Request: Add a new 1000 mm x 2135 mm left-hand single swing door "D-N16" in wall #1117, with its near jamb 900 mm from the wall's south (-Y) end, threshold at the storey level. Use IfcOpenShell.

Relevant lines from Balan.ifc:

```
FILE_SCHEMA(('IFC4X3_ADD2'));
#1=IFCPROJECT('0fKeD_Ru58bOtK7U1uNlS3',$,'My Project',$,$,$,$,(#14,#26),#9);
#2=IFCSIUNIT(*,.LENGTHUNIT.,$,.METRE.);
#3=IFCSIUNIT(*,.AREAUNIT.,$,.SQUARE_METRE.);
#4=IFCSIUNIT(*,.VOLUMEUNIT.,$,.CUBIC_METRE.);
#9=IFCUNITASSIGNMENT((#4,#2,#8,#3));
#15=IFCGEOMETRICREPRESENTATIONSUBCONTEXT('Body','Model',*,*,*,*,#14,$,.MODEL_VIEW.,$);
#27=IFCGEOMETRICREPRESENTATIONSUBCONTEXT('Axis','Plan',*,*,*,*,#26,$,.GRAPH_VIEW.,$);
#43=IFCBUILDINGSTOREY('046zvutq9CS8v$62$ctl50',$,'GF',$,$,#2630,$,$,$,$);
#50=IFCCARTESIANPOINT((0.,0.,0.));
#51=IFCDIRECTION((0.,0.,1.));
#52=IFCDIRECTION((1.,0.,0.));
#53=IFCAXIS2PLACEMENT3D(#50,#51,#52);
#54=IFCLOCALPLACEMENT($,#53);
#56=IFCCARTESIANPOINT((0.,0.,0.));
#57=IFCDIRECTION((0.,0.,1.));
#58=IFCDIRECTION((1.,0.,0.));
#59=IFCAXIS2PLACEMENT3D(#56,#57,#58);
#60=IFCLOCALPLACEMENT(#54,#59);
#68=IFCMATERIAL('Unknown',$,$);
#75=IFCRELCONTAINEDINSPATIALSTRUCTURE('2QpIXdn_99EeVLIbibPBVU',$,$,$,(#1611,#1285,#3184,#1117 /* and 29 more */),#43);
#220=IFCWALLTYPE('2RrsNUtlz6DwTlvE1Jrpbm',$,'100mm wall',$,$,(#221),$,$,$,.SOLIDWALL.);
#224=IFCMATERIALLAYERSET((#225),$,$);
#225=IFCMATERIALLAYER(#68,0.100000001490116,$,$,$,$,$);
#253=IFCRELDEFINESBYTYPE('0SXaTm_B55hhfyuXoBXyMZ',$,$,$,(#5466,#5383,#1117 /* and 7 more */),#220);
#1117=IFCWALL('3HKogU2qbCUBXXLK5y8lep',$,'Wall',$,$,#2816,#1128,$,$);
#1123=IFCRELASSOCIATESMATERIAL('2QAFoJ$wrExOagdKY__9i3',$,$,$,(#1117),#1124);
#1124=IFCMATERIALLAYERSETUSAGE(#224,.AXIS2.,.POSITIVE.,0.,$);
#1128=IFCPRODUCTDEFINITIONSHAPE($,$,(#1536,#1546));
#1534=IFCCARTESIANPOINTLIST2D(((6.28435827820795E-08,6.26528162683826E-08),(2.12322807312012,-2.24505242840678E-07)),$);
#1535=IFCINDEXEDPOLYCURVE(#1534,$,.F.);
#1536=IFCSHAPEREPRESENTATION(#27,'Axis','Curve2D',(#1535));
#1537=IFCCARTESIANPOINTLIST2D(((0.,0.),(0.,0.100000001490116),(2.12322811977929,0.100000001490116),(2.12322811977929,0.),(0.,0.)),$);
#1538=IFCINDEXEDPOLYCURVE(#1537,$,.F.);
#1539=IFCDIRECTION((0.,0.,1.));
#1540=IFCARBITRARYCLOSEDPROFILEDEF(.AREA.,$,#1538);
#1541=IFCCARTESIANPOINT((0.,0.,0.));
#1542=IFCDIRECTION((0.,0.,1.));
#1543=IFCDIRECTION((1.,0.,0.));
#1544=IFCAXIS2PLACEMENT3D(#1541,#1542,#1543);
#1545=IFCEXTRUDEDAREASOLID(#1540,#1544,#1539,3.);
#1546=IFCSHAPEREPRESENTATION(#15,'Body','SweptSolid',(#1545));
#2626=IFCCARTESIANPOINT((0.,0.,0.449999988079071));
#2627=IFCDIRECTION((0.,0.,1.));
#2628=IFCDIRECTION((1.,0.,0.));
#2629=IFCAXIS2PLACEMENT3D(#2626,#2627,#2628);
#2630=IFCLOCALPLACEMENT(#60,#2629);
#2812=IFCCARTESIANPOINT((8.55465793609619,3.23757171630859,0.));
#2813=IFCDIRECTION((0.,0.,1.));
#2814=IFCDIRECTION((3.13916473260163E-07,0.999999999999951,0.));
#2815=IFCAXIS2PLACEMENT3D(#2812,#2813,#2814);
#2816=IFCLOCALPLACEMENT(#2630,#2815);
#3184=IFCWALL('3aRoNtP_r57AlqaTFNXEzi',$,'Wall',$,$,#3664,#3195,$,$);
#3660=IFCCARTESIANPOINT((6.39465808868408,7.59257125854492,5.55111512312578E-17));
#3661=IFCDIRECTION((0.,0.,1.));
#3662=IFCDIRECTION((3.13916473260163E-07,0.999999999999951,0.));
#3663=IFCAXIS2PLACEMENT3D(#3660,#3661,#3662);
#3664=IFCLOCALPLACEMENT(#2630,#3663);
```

```python
import numpy as np
import ifcopenshell
import ifcopenshell.api.feature
import ifcopenshell.api.geometry
import ifcopenshell.api.root
import ifcopenshell.api.spatial
import ifcopenshell.geom
import ifcopenshell.util.element
import ifcopenshell.util.placement
import ifcopenshell.util.representation
import ifcopenshell.util.shape
import ifcopenshell.util.unit

model = ifcopenshell.open("Balan.ifc")
unit_scale = ifcopenshell.util.unit.calculate_unit_scale(model)
settings = ifcopenshell.geom.settings()


def volume(element):
    """Net volume in cubic metres, openings subtracted."""
    shape = ifcopenshell.geom.create_shape(settings, element)
    return ifcopenshell.util.shape.get_volume(shape.geometry)


wall = model.by_guid("3HKogU2qbCUBXXLK5y8lep")
storey = ifcopenshell.util.element.get_container(wall, ifc_class="IfcBuildingStorey")
context = ifcopenshell.util.representation.get_context(model, "Model", "Body", "MODEL_VIEW")
before = volume(wall)

width, height, from_end, sill = 1, 2.135, 0.9, 0.0  # metres

# The wall runs along its own X axis, and the end named is its -X end.
wall_shape = ifcopenshell.geom.create_shape(settings, wall)
x, y, z = ifcopenshell.util.shape.get_vertices(wall_shape.geometry).T
start = x.min() + from_end
face, thickness = float(y.min()), float(y.max() - y.min())
wall_matrix = ifcopenshell.util.placement.get_local_placement(wall.ObjectPlacement)
level = ifcopenshell.util.placement.get_local_placement(storey.ObjectPlacement)[2, 3]


def in_wall(x, y):
    """Placement at x, y metres in the wall's axes, at sill height."""
    matrix = wall_matrix.copy()
    matrix[:, 3] = wall_matrix @ np.array([x / unit_scale, y / unit_scale, 0.0, 1.0])
    matrix[2, 3] = level + sill / unit_scale
    return matrix


# Opening: a box that overshoots both wall faces by 50 mm.
opening = ifcopenshell.api.root.create_entity(model, ifc_class="IfcOpeningElement", predefined_type="OPENING")
box = ifcopenshell.api.geometry.add_wall_representation(
    model, context=context, length=width, height=height, thickness=thickness + 0.1
)
ifcopenshell.api.geometry.assign_representation(model, product=opening, representation=box)
ifcopenshell.api.geometry.edit_object_placement(model, product=opening, matrix=in_wall(start, face - 0.05), is_si=False)
ifcopenshell.api.feature.add_feature(model, feature=opening, element=wall)

door = ifcopenshell.api.root.create_entity(model, ifc_class="IfcDoor", name="D-N16", predefined_type="DOOR")
door.OverallWidth, door.OverallHeight = width / unit_scale, height / unit_scale
door.OperationType = "SINGLE_SWING_LEFT"
body = ifcopenshell.api.geometry.add_door_representation(
    model,
    context=context,
    overall_width=door.OverallWidth,
    overall_height=door.OverallHeight,
    operation_type="SINGLE_SWING_LEFT",
    lining_properties={"LiningDepth": thickness / unit_scale, "ThresholdDepth": thickness / unit_scale},
)
ifcopenshell.api.geometry.assign_representation(model, product=door, representation=body)
ifcopenshell.api.spatial.assign_container(model, products=[door], relating_structure=storey)
ifcopenshell.api.feature.add_filling(model, opening=opening, element=door)

# The lining spans the wall, so the door starts at the wall face.
ifcopenshell.api.geometry.edit_object_placement(model, product=door, matrix=in_wall(start, face), is_si=False)

after = volume(wall)

print(f"wall volume {before:.3f} -> {after:.3f} m3")

model.write("Balan_rev.ifc")
```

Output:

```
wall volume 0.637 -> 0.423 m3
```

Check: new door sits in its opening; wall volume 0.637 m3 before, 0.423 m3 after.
